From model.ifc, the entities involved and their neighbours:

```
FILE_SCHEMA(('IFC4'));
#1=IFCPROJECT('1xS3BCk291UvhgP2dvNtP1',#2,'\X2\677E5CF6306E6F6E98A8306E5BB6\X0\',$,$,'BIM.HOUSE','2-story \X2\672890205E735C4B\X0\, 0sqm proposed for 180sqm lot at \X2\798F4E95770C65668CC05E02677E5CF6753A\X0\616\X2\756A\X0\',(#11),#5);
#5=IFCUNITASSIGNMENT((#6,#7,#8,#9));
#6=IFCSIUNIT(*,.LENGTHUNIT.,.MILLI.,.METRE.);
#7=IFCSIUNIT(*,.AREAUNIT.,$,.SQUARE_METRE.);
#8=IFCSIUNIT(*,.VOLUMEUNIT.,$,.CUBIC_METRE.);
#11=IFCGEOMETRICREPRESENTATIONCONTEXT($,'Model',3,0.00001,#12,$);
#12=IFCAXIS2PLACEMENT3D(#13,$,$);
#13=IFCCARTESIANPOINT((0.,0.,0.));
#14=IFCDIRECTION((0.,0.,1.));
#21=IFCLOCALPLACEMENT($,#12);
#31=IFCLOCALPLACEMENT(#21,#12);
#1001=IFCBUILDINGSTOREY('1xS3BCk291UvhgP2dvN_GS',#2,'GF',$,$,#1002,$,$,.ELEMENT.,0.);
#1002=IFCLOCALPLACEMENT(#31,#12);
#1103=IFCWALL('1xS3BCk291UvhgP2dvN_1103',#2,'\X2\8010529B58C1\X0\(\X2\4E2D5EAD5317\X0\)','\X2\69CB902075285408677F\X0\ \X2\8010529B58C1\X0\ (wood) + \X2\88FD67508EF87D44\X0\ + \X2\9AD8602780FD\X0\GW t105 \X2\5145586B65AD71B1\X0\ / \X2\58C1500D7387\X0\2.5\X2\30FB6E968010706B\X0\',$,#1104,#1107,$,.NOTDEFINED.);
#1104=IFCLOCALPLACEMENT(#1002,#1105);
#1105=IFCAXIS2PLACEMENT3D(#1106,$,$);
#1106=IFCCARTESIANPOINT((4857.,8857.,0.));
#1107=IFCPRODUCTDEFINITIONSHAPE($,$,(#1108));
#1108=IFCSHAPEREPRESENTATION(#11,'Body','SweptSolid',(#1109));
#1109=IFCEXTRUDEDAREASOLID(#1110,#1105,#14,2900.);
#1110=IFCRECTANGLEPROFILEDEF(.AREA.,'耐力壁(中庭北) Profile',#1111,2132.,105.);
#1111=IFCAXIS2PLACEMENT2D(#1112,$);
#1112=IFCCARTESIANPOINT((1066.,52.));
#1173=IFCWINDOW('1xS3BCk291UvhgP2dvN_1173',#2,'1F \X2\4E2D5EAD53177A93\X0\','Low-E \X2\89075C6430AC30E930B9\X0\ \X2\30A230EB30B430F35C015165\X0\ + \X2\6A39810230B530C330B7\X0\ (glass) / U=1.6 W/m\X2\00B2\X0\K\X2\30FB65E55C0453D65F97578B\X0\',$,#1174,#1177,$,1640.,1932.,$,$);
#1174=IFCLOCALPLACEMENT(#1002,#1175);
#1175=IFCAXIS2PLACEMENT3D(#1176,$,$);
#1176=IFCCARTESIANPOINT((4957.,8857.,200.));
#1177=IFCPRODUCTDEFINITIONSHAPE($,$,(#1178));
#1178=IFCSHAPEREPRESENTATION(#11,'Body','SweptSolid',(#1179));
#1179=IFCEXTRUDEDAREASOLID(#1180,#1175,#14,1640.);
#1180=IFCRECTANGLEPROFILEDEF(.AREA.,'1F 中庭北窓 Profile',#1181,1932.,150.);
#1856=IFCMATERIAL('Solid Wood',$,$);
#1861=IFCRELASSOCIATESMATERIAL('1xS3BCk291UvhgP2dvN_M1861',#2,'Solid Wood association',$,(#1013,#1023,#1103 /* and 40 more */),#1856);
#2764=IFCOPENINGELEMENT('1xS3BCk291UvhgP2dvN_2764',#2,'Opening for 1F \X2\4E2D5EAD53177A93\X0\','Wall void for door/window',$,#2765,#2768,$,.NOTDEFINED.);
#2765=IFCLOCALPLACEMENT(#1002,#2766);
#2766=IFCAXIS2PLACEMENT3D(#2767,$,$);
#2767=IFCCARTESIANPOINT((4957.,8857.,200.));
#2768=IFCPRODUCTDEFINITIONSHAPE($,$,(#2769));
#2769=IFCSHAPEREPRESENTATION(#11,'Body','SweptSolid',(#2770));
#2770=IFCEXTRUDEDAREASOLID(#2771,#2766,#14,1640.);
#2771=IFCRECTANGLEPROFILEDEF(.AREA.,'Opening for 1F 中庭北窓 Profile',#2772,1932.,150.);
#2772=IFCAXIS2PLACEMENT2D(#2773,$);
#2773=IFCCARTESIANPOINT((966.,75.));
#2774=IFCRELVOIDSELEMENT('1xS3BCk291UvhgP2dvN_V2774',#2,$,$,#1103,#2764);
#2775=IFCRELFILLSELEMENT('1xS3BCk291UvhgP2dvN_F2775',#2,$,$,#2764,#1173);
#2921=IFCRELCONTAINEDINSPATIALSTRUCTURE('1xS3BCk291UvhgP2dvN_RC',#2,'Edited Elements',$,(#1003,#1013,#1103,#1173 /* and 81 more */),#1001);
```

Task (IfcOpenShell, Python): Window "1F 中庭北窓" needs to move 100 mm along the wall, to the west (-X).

```python
import ifcopenshell
import ifcopenshell.api.geometry
import ifcopenshell.util.placement
import ifcopenshell.util.unit

model = ifcopenshell.open("model.ifc")
unit_scale = ifcopenshell.util.unit.calculate_unit_scale(model)

window = model.by_guid("1xS3BCk291UvhgP2dvN_1173")
opening = window.FillsVoids[0].RelatingOpeningElement
wall = opening.VoidsElements[0].RelatingBuildingElement

wall_matrix = ifcopenshell.util.placement.get_local_placement(wall.ObjectPlacement)
shift = wall_matrix[:3, 0] * -0.1 / unit_scale
before = ifcopenshell.util.placement.get_local_placement(window.ObjectPlacement)[:3, 3].copy()

# The window is not placed relative to its opening, so move both.
for product in (opening, window):
    matrix = ifcopenshell.util.placement.get_local_placement(product.ObjectPlacement)
    matrix[:3, 3] += shift
    ifcopenshell.api.geometry.edit_object_placement(model, product=product, matrix=matrix, is_si=False)

after = ifcopenshell.util.placement.get_local_placement(window.ObjectPlacement)[:3, 3]
print("window moved by", (after - before).round(3) + 0.0)

model.write("model_v2.ifc")
```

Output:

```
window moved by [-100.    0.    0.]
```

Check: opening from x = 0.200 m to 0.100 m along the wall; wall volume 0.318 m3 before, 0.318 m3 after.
